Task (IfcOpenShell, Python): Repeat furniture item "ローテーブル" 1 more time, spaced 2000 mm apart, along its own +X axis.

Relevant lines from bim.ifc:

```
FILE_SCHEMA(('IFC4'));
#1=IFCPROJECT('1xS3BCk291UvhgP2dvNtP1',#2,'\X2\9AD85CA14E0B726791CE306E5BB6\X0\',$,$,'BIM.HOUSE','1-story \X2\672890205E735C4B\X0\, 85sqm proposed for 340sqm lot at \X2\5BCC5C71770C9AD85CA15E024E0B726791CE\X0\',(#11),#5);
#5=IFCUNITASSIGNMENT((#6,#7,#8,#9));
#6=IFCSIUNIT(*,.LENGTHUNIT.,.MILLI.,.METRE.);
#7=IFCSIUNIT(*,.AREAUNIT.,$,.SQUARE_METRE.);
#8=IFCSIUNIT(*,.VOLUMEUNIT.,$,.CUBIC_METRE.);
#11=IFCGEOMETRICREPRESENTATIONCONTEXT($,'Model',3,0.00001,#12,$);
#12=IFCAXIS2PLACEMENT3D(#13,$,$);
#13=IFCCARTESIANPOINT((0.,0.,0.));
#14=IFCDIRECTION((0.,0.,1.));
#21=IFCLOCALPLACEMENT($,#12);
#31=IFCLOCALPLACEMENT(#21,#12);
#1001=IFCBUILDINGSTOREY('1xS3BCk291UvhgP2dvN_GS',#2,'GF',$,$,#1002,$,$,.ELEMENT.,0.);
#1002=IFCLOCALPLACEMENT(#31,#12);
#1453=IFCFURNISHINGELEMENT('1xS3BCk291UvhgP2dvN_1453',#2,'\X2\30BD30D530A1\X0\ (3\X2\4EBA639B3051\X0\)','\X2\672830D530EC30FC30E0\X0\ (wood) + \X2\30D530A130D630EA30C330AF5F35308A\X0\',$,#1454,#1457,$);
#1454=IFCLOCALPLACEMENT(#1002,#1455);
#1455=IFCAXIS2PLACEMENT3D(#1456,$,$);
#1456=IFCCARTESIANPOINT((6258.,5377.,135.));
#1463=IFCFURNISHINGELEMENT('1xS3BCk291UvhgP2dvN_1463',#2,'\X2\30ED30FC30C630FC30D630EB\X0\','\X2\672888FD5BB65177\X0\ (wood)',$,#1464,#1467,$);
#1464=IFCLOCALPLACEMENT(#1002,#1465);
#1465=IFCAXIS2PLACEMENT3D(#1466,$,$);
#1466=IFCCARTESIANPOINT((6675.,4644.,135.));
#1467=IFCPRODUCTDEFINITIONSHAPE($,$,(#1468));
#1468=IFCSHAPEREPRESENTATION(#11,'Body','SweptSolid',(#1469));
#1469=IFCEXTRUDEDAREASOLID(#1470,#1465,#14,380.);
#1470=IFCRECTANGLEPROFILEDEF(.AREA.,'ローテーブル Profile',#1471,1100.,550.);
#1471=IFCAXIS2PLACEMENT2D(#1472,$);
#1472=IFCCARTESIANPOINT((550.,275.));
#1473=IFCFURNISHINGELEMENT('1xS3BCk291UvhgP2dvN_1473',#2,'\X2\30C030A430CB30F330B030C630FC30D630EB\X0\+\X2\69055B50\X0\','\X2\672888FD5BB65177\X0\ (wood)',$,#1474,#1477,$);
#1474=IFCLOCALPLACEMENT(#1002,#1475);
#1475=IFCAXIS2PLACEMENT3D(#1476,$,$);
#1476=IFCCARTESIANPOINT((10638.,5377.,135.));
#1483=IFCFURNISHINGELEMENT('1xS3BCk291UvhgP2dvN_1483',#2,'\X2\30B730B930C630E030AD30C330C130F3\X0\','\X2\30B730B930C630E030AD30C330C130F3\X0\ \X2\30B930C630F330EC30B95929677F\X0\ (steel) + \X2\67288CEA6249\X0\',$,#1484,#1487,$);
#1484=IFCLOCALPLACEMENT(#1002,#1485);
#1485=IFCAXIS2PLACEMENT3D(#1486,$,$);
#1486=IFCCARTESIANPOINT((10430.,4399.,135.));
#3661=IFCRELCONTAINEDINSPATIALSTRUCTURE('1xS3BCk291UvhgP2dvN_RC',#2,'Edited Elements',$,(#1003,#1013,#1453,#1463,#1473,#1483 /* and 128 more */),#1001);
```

```python
import ifcopenshell
import ifcopenshell.api.geometry
import ifcopenshell.api.root
import ifcopenshell.util.element
import ifcopenshell.util.placement

model = ifcopenshell.open("bim.ifc")


def reuse_history(source, copy):
    """copy_class also copies each property set's owner history, people and application; keep the originals."""
    for rel in copy.IsDefinedBy:
        if rel.is_a("IfcRelDefinesByProperties") and (history := rel.RelatingPropertyDefinition.OwnerHistory):
            rel.RelatingPropertyDefinition.OwnerHistory = source.OwnerHistory
            ifcopenshell.util.element.remove_deep2(model, history)


source = model.by_id(1463)
base = ifcopenshell.util.placement.get_local_placement(source.ObjectPlacement)
step = base[:3, 0] * 2000.0

for i in range(1, 2):
    copy = ifcopenshell.api.root.copy_class(model, product=source)
    copy.Representation = ifcopenshell.util.element.copy_deep(
        model, source.Representation, exclude=["IfcGeometricRepresentationContext", "IfcRepresentationMap"]
    )
    reuse_history(source, copy)
    matrix = base.copy()
    matrix[:3, 3] += i * step
    print("added at", matrix[:3, 3].round(3) + 0.0)
    ifcopenshell.api.geometry.edit_object_placement(model, product=copy, matrix=matrix, is_si=False)

model.write("bim_updated.ifc")
```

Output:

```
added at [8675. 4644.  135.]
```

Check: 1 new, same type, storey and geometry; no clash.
